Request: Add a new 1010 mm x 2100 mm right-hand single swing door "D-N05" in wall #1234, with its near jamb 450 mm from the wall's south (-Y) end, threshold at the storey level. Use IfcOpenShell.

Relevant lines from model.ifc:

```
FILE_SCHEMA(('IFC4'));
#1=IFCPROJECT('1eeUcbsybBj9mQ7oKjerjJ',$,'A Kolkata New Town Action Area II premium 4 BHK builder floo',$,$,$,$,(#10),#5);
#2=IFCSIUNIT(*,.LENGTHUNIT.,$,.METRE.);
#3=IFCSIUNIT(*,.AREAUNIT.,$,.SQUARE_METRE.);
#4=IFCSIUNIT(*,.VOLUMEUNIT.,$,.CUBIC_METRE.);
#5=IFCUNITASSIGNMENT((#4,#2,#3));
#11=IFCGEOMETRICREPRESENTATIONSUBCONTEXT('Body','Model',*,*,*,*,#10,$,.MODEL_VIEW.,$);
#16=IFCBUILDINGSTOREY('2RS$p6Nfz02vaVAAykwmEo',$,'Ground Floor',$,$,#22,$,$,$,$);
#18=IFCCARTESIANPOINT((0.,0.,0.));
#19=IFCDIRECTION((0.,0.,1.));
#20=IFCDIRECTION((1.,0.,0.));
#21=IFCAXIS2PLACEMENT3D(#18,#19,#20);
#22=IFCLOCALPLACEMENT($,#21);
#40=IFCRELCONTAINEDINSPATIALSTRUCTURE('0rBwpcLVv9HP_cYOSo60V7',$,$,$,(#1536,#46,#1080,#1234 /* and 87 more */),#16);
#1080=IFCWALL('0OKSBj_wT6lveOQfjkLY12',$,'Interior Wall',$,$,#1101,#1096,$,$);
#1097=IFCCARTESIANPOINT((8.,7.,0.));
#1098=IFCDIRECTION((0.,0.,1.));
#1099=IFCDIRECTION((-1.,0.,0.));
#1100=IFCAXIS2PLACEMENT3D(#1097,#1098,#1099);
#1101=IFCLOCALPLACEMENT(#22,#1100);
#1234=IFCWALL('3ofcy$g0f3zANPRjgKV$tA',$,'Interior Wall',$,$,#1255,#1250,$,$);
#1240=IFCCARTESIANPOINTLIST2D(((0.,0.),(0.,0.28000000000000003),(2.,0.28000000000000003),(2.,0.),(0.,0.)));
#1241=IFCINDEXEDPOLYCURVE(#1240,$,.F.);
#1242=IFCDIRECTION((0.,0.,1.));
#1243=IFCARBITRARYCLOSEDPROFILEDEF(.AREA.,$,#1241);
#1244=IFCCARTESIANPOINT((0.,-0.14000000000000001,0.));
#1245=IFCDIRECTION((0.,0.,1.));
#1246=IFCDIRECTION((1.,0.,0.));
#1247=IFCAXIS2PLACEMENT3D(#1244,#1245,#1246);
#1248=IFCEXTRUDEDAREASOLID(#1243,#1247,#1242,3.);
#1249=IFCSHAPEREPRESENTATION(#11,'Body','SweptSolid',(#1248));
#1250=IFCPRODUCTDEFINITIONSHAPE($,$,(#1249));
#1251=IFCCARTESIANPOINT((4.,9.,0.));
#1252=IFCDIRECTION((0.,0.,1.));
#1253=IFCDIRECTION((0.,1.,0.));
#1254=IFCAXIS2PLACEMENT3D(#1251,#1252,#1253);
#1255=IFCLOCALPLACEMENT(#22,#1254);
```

```python
import numpy as np
import ifcopenshell
import ifcopenshell.api.feature
import ifcopenshell.api.geometry
import ifcopenshell.api.root
import ifcopenshell.api.spatial
import ifcopenshell.geom
import ifcopenshell.util.element
import ifcopenshell.util.placement
import ifcopenshell.util.representation
import ifcopenshell.util.shape
import ifcopenshell.util.unit

model = ifcopenshell.open("model.ifc")
unit_scale = ifcopenshell.util.unit.calculate_unit_scale(model)
settings = ifcopenshell.geom.settings()


def volume(element):
    """Net volume in cubic metres, openings subtracted."""
    shape = ifcopenshell.geom.create_shape(settings, element)
    return ifcopenshell.util.shape.get_volume(shape.geometry)


wall = model.by_guid("3ofcy$g0f3zANPRjgKV$tA")
storey = ifcopenshell.util.element.get_container(wall, ifc_class="IfcBuildingStorey")
context = ifcopenshell.util.representation.get_context(model, "Model", "Body", "MODEL_VIEW")
before = volume(wall)

width, height, from_end, sill = 1.01, 2.1, 0.45, 0.0  # metres

# The wall runs along its own X axis, and the end named is its -X end.
wall_shape = ifcopenshell.geom.create_shape(settings, wall)
x, y, z = ifcopenshell.util.shape.get_vertices(wall_shape.geometry).T
start = x.min() + from_end
face, thickness = float(y.min()), float(y.max() - y.min())
wall_matrix = ifcopenshell.util.placement.get_local_placement(wall.ObjectPlacement)
level = ifcopenshell.util.placement.get_local_placement(storey.ObjectPlacement)[2, 3]


def in_wall(x, y):
    """Placement at x, y metres in the wall's axes, at sill height."""
    matrix = wall_matrix.copy()
    matrix[:, 3] = wall_matrix @ np.array([x / unit_scale, y / unit_scale, 0.0, 1.0])
    matrix[2, 3] = level + sill / unit_scale
    return matrix


# Opening: a box that overshoots both wall faces by 50 mm.
opening = ifcopenshell.api.root.create_entity(model, ifc_class="IfcOpeningElement", predefined_type="OPENING")
box = ifcopenshell.api.geometry.add_wall_representation(
    model, context=context, length=width, height=height, thickness=thickness + 0.1
)
ifcopenshell.api.geometry.assign_representation(model, product=opening, representation=box)
ifcopenshell.api.geometry.edit_object_placement(model, product=opening, matrix=in_wall(start, face - 0.05), is_si=False)
ifcopenshell.api.feature.add_feature(model, feature=opening, element=wall)

door = ifcopenshell.api.root.create_entity(model, ifc_class="IfcDoor", name="D-N05", predefined_type="DOOR")
door.OverallWidth, door.OverallHeight = width / unit_scale, height / unit_scale
door.OperationType = "SINGLE_SWING_RIGHT"
body = ifcopenshell.api.geometry.add_door_representation(
    model,
    context=context,
    overall_width=door.OverallWidth,
    overall_height=door.OverallHeight,
    operation_type="SINGLE_SWING_RIGHT",
    lining_properties={"LiningDepth": thickness / unit_scale, "ThresholdDepth": thickness / unit_scale},
)
ifcopenshell.api.geometry.assign_representation(model, product=door, representation=body)
ifcopenshell.api.spatial.assign_container(model, products=[door], relating_structure=storey)
ifcopenshell.api.feature.add_filling(model, opening=opening, element=door)

# The lining spans the wall, so the door starts at the wall face.
ifcopenshell.api.geometry.edit_object_placement(model, product=door, matrix=in_wall(start, face), is_si=False)

after = volume(wall)

print(f"wall volume {before:.3f} -> {after:.3f} m3")

model.write("model_edited.ifc")
```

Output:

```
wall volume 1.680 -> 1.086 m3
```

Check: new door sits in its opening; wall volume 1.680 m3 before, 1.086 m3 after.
